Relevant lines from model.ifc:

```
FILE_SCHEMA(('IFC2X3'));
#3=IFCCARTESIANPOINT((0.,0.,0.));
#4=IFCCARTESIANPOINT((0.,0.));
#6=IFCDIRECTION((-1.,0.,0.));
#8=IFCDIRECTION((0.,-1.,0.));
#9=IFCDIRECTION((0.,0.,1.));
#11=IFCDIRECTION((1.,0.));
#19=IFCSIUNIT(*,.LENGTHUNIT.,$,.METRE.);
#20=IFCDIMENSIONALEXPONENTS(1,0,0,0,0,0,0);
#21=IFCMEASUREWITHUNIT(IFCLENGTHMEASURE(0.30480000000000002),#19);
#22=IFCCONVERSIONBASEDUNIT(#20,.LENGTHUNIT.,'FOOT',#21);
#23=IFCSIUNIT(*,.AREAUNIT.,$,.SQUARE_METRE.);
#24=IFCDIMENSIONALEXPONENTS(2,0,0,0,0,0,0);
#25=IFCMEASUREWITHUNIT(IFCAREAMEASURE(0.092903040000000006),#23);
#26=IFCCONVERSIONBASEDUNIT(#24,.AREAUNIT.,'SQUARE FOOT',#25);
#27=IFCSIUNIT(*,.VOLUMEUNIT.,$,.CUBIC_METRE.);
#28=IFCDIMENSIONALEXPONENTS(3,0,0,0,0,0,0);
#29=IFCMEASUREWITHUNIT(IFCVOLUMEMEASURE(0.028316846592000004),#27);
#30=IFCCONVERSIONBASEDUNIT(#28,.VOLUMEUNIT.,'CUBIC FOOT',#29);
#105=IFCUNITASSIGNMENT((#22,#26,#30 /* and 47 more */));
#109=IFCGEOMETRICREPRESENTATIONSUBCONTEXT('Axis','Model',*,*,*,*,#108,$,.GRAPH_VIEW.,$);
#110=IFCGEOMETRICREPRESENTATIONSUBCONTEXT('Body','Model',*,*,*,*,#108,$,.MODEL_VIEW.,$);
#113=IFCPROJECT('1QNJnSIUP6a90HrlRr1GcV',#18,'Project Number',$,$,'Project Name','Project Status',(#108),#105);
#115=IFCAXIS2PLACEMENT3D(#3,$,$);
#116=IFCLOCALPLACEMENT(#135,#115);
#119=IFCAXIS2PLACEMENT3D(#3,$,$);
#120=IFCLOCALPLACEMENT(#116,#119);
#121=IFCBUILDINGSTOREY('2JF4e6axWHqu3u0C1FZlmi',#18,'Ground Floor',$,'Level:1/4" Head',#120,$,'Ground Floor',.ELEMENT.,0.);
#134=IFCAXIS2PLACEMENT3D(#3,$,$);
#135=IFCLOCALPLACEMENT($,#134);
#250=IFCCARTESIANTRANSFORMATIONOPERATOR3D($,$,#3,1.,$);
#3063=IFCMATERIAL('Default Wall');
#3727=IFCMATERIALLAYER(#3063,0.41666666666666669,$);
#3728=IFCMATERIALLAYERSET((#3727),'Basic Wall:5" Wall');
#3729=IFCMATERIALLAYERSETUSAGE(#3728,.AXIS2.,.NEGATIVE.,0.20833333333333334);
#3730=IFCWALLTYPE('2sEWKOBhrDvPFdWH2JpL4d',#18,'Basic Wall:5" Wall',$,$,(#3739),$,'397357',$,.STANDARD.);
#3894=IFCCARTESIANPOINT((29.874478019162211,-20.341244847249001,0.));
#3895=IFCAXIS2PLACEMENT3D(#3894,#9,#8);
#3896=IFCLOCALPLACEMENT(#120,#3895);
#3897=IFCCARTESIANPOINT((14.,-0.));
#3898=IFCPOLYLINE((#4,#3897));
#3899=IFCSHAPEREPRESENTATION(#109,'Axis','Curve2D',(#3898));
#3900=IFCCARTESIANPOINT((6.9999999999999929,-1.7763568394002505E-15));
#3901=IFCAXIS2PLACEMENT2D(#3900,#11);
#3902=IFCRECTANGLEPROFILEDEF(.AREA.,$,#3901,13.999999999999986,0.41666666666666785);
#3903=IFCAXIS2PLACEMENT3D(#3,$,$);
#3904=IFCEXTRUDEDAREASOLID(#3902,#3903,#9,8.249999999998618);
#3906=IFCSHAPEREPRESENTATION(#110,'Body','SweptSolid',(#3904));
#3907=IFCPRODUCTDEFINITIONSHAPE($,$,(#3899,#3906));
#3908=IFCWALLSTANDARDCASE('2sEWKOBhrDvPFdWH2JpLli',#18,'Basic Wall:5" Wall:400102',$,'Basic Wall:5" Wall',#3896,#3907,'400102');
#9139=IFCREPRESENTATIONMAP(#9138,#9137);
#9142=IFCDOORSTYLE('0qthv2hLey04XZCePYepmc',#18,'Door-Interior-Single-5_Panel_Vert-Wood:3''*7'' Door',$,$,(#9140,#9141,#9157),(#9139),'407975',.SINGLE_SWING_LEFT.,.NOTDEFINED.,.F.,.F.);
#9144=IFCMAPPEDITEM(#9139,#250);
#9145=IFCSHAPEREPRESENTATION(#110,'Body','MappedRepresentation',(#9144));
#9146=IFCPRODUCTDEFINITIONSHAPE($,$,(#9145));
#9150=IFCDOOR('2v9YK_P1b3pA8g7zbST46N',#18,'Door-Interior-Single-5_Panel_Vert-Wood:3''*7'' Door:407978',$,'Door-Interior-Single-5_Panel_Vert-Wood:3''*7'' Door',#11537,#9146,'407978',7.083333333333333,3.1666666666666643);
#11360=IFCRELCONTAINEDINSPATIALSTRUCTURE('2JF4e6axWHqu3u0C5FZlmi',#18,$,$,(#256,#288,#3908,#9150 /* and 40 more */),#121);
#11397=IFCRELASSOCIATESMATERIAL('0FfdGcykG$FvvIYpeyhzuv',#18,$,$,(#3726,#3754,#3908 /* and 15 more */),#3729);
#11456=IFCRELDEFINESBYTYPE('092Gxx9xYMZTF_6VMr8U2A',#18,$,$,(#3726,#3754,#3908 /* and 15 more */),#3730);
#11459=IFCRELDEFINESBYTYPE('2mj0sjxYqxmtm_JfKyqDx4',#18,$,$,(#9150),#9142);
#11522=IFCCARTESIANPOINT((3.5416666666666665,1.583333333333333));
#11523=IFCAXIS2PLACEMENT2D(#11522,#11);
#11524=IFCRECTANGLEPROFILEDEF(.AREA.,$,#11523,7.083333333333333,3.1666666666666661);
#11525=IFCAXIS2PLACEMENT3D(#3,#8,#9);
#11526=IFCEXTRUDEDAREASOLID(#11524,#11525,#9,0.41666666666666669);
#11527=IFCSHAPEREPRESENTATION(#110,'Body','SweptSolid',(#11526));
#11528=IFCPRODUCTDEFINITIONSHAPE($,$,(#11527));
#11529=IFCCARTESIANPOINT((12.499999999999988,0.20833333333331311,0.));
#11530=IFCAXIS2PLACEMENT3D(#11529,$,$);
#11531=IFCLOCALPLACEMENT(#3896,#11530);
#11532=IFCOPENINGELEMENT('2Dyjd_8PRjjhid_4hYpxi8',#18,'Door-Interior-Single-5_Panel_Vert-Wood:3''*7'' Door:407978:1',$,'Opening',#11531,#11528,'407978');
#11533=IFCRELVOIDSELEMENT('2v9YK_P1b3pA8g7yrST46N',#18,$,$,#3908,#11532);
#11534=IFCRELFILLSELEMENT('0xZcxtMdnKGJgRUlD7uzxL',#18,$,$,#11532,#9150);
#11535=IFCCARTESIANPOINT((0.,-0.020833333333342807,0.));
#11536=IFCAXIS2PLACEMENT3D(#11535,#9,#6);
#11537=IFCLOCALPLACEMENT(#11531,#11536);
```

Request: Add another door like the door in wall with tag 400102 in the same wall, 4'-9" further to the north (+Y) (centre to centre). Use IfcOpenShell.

```python
import ifcopenshell
import ifcopenshell.api.feature
import ifcopenshell.api.geometry
import ifcopenshell.api.root
import ifcopenshell.geom
import ifcopenshell.util.element
import ifcopenshell.util.placement
import ifcopenshell.util.shape
import ifcopenshell.util.unit

model = ifcopenshell.open("model.ifc")
unit_scale = ifcopenshell.util.unit.calculate_unit_scale(model)
settings = ifcopenshell.geom.settings()


def volume(element):
    """Net volume in cubic metres, openings subtracted."""
    shape = ifcopenshell.geom.create_shape(settings, element)
    return ifcopenshell.util.shape.get_volume(shape.geometry)


def reuse_history(source, copy):
    """copy_class also copies each property set's owner history, people and application; keep the originals."""
    for rel in copy.IsDefinedBy:
        if rel.is_a("IfcRelDefinesByProperties") and (history := rel.RelatingPropertyDefinition.OwnerHistory):
            rel.RelatingPropertyDefinition.OwnerHistory = source.OwnerHistory
            ifcopenshell.util.element.remove_deep2(model, history)


door = model.by_id(9150)
opening = door.FillsVoids[0].RelatingOpeningElement
wall = opening.VoidsElements[0].RelatingBuildingElement
before = volume(wall)
shift = ifcopenshell.util.placement.get_local_placement(wall.ObjectPlacement)[:3, 0] * -57 * 0.0254 / unit_scale

# copy_class copies the void relationship, type, container and properties, but no geometry.
new_opening = ifcopenshell.api.root.copy_class(model, product=opening)
new_opening.Representation = ifcopenshell.util.element.copy_deep(
    model, opening.Representation, exclude=["IfcGeometricRepresentationContext", "IfcRepresentationMap"]
)
new_opening.Name = "Door-Interior-Single-5_Panel_Vert-Wood:3'*7' Door"
new_opening.Tag = None
new_door = ifcopenshell.api.root.copy_class(model, product=door)
new_door.Representation = ifcopenshell.util.element.copy_deep(
    model, door.Representation, exclude=["IfcGeometricRepresentationContext", "IfcRepresentationMap"]
)
new_door.Name = "Door-Interior-Single-5_Panel_Vert-Wood:3'*7' Door"
new_door.Tag = None
reuse_history(door, new_door)
fills = ifcopenshell.api.feature.add_filling(model, opening=new_opening, element=new_door)
fills.OwnerHistory = new_door.OwnerHistory  # required in IFC2X3

for old, new in ((opening, new_opening), (door, new_door)):
    matrix = ifcopenshell.util.placement.get_local_placement(old.ObjectPlacement)
    matrix[:3, 3] += shift
    ifcopenshell.api.geometry.edit_object_placement(model, product=new, matrix=matrix, is_si=False)

after = volume(wall)

print(f"wall volume {before:.3f} -> {after:.3f} m3")

model.write("model_edited.ifc")
```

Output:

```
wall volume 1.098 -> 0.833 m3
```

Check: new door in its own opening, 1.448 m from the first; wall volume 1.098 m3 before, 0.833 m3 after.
